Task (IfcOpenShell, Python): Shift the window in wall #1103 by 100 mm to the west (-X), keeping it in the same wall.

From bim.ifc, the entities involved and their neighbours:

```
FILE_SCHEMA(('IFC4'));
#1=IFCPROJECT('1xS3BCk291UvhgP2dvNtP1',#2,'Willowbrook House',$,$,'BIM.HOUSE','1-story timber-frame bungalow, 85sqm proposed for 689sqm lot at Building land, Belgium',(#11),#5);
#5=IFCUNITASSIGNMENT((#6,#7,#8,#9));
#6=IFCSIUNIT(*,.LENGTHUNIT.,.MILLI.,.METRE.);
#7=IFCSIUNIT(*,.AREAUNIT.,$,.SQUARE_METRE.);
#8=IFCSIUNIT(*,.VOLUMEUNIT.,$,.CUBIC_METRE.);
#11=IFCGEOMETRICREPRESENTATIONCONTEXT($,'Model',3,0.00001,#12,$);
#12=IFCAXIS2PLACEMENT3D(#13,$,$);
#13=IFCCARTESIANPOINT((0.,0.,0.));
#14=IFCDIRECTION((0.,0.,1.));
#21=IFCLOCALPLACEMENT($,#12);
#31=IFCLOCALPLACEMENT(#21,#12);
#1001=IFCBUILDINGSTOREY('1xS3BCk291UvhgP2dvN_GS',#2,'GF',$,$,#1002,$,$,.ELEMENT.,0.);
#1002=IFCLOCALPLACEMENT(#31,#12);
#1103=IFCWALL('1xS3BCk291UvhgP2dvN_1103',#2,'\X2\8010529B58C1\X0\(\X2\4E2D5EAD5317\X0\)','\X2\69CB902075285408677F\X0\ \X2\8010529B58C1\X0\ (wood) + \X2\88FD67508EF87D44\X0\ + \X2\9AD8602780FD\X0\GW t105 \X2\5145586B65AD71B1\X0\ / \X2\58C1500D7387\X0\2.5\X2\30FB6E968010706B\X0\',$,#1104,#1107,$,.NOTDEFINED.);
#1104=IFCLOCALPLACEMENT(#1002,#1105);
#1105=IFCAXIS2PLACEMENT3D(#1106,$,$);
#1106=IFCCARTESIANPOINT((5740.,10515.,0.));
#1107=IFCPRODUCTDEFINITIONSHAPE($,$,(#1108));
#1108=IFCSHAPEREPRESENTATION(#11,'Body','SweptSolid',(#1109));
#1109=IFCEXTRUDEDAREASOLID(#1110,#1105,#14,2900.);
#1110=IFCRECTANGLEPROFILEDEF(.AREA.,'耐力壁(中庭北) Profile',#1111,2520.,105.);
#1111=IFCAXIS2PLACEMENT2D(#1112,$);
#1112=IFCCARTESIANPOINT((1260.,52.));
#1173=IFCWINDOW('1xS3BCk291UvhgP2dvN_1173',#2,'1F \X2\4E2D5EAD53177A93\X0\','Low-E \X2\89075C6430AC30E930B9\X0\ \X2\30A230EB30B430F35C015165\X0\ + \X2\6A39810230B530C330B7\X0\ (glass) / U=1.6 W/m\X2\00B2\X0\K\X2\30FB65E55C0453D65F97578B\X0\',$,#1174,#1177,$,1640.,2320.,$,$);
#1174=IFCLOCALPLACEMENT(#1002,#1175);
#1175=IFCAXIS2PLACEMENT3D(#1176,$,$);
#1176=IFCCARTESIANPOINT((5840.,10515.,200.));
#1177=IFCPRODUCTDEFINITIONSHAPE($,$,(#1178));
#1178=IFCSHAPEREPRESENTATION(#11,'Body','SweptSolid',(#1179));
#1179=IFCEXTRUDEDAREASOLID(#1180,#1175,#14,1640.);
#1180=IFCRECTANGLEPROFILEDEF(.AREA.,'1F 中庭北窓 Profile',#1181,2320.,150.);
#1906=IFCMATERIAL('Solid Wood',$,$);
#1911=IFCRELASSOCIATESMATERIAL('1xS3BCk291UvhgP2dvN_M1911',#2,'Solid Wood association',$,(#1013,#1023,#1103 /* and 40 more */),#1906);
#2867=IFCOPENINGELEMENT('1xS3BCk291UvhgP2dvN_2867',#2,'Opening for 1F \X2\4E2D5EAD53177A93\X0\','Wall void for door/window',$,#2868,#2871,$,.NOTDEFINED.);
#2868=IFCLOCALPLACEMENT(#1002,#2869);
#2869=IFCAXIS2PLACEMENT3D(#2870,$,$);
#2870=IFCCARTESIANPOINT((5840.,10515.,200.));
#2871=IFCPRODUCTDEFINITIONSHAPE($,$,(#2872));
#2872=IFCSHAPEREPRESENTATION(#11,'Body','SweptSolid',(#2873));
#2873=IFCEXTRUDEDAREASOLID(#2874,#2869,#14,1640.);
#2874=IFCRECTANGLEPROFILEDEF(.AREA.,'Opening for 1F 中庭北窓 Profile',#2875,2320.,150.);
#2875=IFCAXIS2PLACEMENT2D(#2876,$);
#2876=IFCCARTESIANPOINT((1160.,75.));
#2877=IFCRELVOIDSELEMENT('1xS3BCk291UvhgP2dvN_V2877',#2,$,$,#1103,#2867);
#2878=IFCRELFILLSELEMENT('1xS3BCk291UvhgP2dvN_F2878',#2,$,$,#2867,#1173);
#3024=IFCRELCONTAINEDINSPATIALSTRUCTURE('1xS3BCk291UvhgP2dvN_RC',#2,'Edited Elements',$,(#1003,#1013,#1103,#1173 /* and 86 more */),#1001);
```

```python
import ifcopenshell
import ifcopenshell.api.geometry
import ifcopenshell.util.placement

model = ifcopenshell.open("bim.ifc")

window = model.by_guid("1xS3BCk291UvhgP2dvN_1173")
opening = window.FillsVoids[0].RelatingOpeningElement
wall = opening.VoidsElements[0].RelatingBuildingElement

wall_matrix = ifcopenshell.util.placement.get_local_placement(wall.ObjectPlacement)
shift = wall_matrix[:3, 0] * -100.0
before = ifcopenshell.util.placement.get_local_placement(window.ObjectPlacement)[:3, 3].copy()

# The window is not placed relative to its opening, so move both.
for product in (opening, window):
    matrix = ifcopenshell.util.placement.get_local_placement(product.ObjectPlacement)
    matrix[:3, 3] += shift
    ifcopenshell.api.geometry.edit_object_placement(model, product=product, matrix=matrix, is_si=False)

after = ifcopenshell.util.placement.get_local_placement(window.ObjectPlacement)[:3, 3]
print("window moved by", (after - before).round(3) + 0.0)

model.write("bim_edited.ifc")
```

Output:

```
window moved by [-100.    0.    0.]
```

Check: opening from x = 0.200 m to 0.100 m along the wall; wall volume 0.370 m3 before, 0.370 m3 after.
